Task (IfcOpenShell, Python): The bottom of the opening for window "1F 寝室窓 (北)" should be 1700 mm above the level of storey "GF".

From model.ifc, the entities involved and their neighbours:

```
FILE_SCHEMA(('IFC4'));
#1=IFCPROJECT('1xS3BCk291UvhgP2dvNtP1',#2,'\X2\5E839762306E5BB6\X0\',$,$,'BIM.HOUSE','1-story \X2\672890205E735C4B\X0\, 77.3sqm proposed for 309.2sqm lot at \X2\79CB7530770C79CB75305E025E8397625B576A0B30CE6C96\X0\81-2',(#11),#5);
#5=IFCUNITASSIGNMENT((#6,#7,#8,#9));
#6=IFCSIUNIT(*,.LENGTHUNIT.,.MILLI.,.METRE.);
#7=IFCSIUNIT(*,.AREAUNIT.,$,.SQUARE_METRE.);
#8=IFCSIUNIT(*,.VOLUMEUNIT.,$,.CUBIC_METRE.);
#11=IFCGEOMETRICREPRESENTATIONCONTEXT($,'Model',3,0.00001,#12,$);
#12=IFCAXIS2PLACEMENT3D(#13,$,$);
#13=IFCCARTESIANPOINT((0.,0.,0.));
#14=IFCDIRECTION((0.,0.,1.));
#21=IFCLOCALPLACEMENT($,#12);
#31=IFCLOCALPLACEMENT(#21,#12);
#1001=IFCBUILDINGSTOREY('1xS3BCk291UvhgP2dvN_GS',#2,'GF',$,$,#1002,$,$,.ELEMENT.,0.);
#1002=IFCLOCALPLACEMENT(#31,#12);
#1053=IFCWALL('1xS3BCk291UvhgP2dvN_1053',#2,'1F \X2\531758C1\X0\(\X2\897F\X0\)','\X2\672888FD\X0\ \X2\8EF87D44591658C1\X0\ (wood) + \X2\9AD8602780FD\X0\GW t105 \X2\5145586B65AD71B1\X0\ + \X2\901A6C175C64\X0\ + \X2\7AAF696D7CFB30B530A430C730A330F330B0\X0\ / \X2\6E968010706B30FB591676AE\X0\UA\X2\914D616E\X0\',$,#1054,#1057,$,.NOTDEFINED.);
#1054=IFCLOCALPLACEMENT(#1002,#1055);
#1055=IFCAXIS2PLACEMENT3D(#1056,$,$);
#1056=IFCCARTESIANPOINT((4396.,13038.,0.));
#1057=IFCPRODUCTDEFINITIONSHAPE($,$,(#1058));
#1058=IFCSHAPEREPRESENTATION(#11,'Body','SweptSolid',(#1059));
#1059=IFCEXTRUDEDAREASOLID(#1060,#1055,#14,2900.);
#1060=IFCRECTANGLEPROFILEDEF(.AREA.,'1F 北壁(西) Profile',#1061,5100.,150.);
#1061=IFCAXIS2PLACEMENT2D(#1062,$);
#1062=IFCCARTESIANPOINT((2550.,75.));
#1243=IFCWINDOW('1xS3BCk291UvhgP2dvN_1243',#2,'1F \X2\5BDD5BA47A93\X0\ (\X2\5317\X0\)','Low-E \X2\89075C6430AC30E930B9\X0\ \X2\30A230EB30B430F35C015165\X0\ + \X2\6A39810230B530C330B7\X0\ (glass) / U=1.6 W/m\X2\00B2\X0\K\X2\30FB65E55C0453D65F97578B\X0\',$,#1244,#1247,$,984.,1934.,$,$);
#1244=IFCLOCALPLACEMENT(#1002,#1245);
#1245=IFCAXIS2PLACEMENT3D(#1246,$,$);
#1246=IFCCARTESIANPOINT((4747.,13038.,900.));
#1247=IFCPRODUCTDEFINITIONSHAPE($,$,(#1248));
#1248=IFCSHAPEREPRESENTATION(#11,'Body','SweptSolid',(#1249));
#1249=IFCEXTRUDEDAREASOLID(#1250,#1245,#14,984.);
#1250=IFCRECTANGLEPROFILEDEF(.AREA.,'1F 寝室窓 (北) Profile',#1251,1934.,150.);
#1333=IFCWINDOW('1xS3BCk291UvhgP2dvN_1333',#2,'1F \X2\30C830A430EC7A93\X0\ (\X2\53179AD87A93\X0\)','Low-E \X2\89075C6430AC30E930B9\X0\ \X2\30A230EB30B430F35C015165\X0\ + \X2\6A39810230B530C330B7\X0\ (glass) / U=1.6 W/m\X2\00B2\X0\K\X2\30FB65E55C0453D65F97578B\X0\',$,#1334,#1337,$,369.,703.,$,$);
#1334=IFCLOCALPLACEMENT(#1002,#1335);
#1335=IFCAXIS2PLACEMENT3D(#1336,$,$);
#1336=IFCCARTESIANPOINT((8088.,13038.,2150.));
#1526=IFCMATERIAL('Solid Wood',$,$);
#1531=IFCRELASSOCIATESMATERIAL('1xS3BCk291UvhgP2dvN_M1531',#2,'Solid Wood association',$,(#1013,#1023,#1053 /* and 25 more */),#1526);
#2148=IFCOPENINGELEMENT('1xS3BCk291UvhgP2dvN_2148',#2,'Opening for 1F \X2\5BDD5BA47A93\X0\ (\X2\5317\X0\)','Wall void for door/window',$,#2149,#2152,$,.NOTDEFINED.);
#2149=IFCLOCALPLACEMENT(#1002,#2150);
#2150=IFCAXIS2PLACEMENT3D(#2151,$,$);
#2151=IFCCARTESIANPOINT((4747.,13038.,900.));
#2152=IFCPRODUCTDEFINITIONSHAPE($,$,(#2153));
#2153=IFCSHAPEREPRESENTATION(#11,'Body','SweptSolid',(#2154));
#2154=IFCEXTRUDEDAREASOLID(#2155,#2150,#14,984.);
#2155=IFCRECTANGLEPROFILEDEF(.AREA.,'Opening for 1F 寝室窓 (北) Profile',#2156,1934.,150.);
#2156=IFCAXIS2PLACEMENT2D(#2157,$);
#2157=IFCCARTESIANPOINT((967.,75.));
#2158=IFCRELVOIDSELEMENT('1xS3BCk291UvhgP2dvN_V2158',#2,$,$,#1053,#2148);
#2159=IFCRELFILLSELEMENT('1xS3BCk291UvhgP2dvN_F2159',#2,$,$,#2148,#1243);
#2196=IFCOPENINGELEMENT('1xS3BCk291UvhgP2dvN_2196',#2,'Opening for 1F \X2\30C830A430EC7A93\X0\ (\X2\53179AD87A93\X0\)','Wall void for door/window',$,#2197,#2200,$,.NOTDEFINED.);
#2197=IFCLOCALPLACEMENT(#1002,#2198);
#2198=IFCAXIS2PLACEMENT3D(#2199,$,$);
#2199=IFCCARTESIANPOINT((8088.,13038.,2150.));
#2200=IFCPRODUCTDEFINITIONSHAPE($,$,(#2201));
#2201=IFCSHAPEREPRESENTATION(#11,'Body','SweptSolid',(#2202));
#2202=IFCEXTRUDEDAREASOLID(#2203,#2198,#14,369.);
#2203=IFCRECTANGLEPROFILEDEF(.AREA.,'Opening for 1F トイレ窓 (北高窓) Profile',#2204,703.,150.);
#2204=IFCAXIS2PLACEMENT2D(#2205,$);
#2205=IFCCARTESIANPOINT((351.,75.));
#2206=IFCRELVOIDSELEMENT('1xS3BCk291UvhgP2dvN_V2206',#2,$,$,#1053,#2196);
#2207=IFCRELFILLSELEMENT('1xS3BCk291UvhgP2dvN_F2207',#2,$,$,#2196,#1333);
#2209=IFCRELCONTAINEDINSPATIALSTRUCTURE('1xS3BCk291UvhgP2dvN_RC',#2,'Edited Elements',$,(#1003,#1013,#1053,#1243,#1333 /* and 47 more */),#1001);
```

```python
import numpy as np
import ifcopenshell
import ifcopenshell.api.geometry
import ifcopenshell.geom
import ifcopenshell.util.element
import ifcopenshell.util.placement
import ifcopenshell.util.shape
import ifcopenshell.util.unit

model = ifcopenshell.open("model.ifc")
unit_scale = ifcopenshell.util.unit.calculate_unit_scale(model)

window = model.by_guid("1xS3BCk291UvhgP2dvN_1243")
opening = window.FillsVoids[0].RelatingOpeningElement
storey = ifcopenshell.util.element.get_container(window, ifc_class="IfcBuildingStorey")
level = ifcopenshell.util.placement.get_local_placement(storey.ObjectPlacement)[2, 3]

# The opening's origin need not be at the sill, so measure its lowest point.
shape = ifcopenshell.geom.create_shape(ifcopenshell.geom.settings(), opening)
bottom = ifcopenshell.util.shape.get_shape_bottom_elevation(shape, shape.geometry) / unit_scale
dz = level + 1700.0 - bottom

shift = np.array([0.0, 0.0, dz])
# The window is not placed relative to its opening, so move both.
for product in (opening, window):
    matrix = ifcopenshell.util.placement.get_local_placement(product.ObjectPlacement)
    matrix[:3, 3] += shift
    ifcopenshell.api.geometry.edit_object_placement(model, product=product, matrix=matrix, is_si=False)

print(f"moved by {dz * unit_scale:+.3f} m")

model.write("model_rev.ifc")
```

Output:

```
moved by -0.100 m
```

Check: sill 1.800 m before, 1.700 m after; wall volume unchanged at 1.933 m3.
